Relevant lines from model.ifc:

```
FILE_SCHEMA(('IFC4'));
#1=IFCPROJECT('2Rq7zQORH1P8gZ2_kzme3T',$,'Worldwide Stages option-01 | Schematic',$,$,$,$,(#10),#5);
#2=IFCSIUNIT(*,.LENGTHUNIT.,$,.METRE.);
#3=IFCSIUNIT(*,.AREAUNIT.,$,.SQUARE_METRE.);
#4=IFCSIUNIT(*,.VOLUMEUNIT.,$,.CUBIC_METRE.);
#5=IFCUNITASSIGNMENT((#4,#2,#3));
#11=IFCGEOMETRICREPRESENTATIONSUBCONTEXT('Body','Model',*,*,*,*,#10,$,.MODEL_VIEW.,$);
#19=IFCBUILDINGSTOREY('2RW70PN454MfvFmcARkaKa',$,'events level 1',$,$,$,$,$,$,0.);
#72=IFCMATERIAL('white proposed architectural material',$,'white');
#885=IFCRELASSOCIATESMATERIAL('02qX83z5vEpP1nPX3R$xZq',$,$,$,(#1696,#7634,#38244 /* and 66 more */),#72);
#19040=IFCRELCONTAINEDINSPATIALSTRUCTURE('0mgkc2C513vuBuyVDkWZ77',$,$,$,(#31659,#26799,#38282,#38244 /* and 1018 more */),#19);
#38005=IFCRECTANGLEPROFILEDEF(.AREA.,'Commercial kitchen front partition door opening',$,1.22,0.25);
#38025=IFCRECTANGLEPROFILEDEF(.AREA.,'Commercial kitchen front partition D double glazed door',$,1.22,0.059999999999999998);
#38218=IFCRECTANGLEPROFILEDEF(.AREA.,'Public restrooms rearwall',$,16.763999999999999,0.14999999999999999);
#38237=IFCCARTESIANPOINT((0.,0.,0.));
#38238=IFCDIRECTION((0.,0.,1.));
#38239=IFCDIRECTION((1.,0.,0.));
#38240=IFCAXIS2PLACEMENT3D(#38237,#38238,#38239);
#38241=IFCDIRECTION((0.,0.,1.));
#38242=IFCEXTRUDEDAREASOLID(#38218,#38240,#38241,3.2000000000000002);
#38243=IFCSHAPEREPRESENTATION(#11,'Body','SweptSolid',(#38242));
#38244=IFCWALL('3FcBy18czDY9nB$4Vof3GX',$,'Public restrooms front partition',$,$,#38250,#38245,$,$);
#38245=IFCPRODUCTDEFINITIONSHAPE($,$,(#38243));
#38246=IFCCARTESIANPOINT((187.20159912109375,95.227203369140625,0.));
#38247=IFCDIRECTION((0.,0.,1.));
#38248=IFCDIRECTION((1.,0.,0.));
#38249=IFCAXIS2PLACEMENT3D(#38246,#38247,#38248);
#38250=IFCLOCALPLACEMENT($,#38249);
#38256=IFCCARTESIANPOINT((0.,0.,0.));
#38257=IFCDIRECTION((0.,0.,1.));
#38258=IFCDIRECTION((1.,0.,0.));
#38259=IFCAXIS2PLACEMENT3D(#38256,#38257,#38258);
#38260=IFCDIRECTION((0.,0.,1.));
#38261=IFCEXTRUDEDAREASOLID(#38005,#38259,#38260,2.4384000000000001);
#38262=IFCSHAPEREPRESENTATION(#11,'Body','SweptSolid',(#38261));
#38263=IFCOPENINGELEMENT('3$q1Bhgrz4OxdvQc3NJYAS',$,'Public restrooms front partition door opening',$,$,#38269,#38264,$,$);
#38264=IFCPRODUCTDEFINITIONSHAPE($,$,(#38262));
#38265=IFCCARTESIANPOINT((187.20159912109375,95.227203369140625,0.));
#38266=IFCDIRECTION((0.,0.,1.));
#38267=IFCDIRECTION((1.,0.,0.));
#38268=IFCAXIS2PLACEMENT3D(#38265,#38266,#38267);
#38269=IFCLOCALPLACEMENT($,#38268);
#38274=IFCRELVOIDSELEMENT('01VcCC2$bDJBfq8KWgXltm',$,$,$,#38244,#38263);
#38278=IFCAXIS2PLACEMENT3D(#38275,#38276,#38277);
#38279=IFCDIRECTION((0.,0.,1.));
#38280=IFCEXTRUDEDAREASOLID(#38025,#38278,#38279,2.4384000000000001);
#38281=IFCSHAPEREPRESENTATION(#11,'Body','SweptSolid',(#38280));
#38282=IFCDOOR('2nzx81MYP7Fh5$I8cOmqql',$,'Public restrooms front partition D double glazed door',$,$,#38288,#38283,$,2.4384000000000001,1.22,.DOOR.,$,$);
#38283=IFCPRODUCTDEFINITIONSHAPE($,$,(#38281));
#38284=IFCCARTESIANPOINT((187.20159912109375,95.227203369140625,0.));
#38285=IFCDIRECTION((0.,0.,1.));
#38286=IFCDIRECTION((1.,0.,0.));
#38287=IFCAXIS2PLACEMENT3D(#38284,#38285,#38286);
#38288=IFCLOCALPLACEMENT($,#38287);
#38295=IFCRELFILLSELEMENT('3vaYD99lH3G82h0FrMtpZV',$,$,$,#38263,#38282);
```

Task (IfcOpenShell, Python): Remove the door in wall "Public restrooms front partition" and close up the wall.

```python
import ifcopenshell
import ifcopenshell.api.feature
import ifcopenshell.api.root
import ifcopenshell.geom
import ifcopenshell.util.shape

model = ifcopenshell.open("model.ifc")
settings = ifcopenshell.geom.settings()


def volume(element):
    """Net volume in cubic metres, openings subtracted."""
    shape = ifcopenshell.geom.create_shape(settings, element)
    return ifcopenshell.util.shape.get_volume(shape.geometry)


door = model.by_guid("2nzx81MYP7Fh5$I8cOmqql")
opening = door.FillsVoids[0].RelatingOpeningElement
wall = opening.VoidsElements[0].RelatingBuildingElement
before = volume(wall)

ifcopenshell.api.root.remove_product(model, product=door)
ifcopenshell.api.feature.remove_feature(model, feature=opening)

after = volume(wall)

print(f"wall volume {before:.3f} -> {after:.3f} m3")

model.write("model_edited.ifc")
```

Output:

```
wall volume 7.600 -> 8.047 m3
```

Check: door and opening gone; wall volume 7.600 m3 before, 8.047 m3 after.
